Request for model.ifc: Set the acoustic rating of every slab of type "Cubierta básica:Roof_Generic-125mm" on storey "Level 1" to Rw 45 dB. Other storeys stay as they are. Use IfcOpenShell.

First a look at what the model holds.

```python
import ifcopenshell
import ifcopenshell.util.element

model = ifcopenshell.open("model.ifc")
print(model.schema)
storey = next(s for s in model.by_type("IfcBuildingStorey") if s.Name == "Level 1")
slabs = [e for e in ifcopenshell.util.element.get_decomposition(storey) if e.is_a("IfcSlab")]
seen = {}
for e in slabs:
    element_type = ifcopenshell.util.element.get_type(e)
    key = (element_type.Name if element_type != e and element_type else None, ifcopenshell.util.element.get_pset(e, "Pset_SlabCommon", "AcousticRating"))
    seen[key] = seen.get(key, 0) + 1
for (name, value), count in sorted(seen.items(), key=str):
    print(count, "x", name, "|", value)
```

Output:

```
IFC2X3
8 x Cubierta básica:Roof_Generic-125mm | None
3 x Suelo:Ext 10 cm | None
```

```python
import ifcopenshell
import ifcopenshell.api.pset
import ifcopenshell.util.element

model = ifcopenshell.open("model.ifc")

storey = next(s for s in model.by_type("IfcBuildingStorey") if s.Name == "Level 1")
slabs = [e for e in ifcopenshell.util.element.get_decomposition(storey) if e.is_a("IfcSlab")]

count = 0
for e in slabs:
    element_type = ifcopenshell.util.element.get_type(e)
    if element_type in (None, e) or element_type.Name != "Cubierta básica:Roof_Generic-125mm":
        continue
    # add_pset returns the element's existing set when there is one.
    pset = ifcopenshell.api.pset.add_pset(model, product=e, name="Pset_SlabCommon")
    ifcopenshell.api.pset.edit_pset(model, pset=pset, properties={"AcousticRating": "Rw 45 dB"})
    count += 1

print(count, "slabs updated")

model.write("model_v2.ifc")
```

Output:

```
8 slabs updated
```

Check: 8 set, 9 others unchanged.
